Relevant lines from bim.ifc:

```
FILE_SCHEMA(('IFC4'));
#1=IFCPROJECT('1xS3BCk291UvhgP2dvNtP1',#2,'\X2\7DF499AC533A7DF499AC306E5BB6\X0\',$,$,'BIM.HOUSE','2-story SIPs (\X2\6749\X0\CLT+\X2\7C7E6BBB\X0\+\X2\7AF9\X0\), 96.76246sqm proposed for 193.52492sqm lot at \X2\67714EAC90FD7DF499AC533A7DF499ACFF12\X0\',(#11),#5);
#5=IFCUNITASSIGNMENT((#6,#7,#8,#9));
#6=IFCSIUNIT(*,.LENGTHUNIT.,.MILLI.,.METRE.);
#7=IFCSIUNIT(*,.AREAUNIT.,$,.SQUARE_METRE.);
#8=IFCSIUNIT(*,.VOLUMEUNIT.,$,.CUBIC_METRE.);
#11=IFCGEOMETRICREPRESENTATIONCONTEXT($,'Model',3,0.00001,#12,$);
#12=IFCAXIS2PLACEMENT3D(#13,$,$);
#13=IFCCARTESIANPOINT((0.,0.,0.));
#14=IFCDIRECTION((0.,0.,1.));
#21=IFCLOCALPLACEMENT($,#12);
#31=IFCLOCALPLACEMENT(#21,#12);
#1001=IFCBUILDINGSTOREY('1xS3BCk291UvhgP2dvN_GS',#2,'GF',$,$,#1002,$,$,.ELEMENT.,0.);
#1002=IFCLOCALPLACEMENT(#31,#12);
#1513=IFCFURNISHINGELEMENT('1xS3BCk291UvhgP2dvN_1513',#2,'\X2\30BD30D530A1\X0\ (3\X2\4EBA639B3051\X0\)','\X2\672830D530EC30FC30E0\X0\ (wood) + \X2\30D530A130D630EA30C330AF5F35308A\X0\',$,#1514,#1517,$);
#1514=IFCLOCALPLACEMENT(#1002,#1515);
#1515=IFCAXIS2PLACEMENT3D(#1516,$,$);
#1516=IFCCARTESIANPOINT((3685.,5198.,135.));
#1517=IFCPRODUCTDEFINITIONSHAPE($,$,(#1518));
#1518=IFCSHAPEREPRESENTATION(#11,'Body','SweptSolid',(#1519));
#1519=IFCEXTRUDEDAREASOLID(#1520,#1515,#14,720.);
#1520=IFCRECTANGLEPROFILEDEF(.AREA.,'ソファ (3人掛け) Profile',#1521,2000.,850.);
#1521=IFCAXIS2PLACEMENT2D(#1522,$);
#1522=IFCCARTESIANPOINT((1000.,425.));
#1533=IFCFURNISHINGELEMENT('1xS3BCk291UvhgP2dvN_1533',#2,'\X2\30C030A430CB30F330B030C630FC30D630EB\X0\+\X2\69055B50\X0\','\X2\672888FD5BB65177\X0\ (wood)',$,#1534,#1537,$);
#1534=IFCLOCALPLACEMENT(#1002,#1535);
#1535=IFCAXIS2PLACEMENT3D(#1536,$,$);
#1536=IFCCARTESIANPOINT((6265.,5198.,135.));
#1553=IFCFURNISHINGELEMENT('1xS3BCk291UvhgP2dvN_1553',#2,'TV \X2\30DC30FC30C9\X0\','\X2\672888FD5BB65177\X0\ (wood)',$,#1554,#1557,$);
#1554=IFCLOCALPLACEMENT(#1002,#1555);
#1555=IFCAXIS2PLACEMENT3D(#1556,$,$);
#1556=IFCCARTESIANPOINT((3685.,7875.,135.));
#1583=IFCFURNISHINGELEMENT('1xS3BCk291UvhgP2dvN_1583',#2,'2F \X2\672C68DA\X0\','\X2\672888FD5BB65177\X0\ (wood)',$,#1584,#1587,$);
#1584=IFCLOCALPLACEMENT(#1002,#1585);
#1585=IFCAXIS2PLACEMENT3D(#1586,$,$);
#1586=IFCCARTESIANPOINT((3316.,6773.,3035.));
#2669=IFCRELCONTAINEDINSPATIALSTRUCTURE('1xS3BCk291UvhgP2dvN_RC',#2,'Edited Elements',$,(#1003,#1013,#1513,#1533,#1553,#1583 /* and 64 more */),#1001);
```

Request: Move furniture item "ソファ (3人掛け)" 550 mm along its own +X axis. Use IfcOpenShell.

```python
import ifcopenshell
import ifcopenshell.api.geometry
import ifcopenshell.util.placement
import ifcopenshell.util.unit

model = ifcopenshell.open("bim.ifc")
unit_scale = ifcopenshell.util.unit.calculate_unit_scale(model)

item = model.by_guid("1xS3BCk291UvhgP2dvN_1513")
matrix = ifcopenshell.util.placement.get_local_placement(item.ObjectPlacement)
matrix[:3, 3] += matrix[:3, 0] * 0.55 / unit_scale
ifcopenshell.api.geometry.edit_object_placement(model, product=item, matrix=matrix, is_si=False)

print(ifcopenshell.util.placement.get_local_placement(item.ObjectPlacement).round(3) + 0.0)

model.write("bim_rev.ifc")
```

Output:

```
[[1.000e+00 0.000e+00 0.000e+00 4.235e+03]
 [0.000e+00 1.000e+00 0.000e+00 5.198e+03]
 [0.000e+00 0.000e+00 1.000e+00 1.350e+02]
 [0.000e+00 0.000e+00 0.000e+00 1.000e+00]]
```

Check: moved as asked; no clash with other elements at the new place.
